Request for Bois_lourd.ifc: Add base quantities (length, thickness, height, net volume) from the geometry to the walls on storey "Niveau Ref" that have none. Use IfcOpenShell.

First a look at what the model holds.

```python
import ifcopenshell
import ifcopenshell.util.element
import ifcopenshell.util.unit

model = ifcopenshell.open("Bois_lourd.ifc")
print(model.schema)
for unit_type in ("LENGTHUNIT", "AREAUNIT", "VOLUMEUNIT"):
    print(unit_type, ifcopenshell.util.unit.calculate_unit_scale(model, unit_type))
storey = next(s for s in model.by_type("IfcBuildingStorey") if s.Name == "Niveau Ref")
walls = [e for e in ifcopenshell.util.element.get_decomposition(storey) if e.is_a("IfcWall")]
for e in sorted(walls, key=lambda e: e.id()):
    print(e.id(), e.is_a(), e.Name, list(ifcopenshell.util.element.get_psets(e, qtos_only=True)), sep=" | ")
```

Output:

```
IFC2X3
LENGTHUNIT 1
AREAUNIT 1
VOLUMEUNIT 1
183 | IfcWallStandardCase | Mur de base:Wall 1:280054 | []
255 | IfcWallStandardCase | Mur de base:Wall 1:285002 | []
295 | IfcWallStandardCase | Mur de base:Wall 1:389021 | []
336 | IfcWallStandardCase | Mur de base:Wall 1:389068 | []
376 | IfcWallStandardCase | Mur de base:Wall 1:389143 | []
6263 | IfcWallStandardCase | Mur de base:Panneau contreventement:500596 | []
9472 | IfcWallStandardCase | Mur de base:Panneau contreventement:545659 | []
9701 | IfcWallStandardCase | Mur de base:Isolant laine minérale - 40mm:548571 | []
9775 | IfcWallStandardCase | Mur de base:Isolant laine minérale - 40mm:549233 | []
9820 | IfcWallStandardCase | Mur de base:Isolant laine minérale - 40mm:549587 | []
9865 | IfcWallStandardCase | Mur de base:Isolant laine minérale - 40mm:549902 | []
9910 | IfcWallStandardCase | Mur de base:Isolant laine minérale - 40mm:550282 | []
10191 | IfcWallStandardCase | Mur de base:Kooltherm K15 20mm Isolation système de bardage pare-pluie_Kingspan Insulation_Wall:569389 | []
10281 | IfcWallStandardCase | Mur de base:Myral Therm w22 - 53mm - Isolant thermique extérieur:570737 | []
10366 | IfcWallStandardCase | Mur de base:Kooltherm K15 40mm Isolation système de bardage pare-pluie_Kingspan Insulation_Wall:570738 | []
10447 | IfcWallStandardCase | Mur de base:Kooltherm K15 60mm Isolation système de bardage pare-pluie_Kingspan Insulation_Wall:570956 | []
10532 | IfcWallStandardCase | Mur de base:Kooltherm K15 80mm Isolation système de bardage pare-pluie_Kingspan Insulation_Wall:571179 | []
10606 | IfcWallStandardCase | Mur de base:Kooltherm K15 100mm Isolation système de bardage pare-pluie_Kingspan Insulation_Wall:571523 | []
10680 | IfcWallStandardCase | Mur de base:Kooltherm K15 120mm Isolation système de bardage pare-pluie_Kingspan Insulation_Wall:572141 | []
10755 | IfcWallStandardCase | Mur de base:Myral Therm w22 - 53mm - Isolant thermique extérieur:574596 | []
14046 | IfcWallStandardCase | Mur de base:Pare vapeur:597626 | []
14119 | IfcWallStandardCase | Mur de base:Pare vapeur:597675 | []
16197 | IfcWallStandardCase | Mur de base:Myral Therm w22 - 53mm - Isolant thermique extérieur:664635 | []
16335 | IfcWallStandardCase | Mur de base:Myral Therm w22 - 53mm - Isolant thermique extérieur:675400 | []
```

```python
import ifcopenshell
import ifcopenshell.api.pset
import ifcopenshell.geom
import ifcopenshell.util.element
import ifcopenshell.util.shape
import ifcopenshell.util.unit

model = ifcopenshell.open("Bois_lourd.ifc")
unit_scale = ifcopenshell.util.unit.calculate_unit_scale(model)
volume_scale = ifcopenshell.util.unit.calculate_unit_scale(model, "VOLUMEUNIT")
settings = ifcopenshell.geom.settings()

storey = next(s for s in model.by_type("IfcBuildingStorey") if s.Name == "Niveau Ref")
walls = [e for e in ifcopenshell.util.element.get_decomposition(storey) if e.is_a("IfcWall")]

for e in sorted(walls, key=lambda e: e.id()):
    if ifcopenshell.util.element.get_psets(e, qtos_only=True, should_inherit=False):
        continue
    # Geometry comes back in metres, in the element's own axes.
    shape = ifcopenshell.geom.create_shape(settings, e)
    values = {
        "Length": ifcopenshell.util.shape.get_x(shape.geometry) / unit_scale,
        "Width": ifcopenshell.util.shape.get_y(shape.geometry) / unit_scale,
        "Height": ifcopenshell.util.shape.get_z(shape.geometry) / unit_scale,
        "NetVolume": ifcopenshell.util.shape.get_volume(shape.geometry) / volume_scale,
    }
    qto = ifcopenshell.api.pset.add_qto(model, product=e, name="BaseQuantities")
    ifcopenshell.api.pset.edit_qto(model, qto=qto, properties=values)
    print(e.id(), {k: round(v, 3) for k, v in values.items()})

model.write("Bois_lourd-out.ifc")
```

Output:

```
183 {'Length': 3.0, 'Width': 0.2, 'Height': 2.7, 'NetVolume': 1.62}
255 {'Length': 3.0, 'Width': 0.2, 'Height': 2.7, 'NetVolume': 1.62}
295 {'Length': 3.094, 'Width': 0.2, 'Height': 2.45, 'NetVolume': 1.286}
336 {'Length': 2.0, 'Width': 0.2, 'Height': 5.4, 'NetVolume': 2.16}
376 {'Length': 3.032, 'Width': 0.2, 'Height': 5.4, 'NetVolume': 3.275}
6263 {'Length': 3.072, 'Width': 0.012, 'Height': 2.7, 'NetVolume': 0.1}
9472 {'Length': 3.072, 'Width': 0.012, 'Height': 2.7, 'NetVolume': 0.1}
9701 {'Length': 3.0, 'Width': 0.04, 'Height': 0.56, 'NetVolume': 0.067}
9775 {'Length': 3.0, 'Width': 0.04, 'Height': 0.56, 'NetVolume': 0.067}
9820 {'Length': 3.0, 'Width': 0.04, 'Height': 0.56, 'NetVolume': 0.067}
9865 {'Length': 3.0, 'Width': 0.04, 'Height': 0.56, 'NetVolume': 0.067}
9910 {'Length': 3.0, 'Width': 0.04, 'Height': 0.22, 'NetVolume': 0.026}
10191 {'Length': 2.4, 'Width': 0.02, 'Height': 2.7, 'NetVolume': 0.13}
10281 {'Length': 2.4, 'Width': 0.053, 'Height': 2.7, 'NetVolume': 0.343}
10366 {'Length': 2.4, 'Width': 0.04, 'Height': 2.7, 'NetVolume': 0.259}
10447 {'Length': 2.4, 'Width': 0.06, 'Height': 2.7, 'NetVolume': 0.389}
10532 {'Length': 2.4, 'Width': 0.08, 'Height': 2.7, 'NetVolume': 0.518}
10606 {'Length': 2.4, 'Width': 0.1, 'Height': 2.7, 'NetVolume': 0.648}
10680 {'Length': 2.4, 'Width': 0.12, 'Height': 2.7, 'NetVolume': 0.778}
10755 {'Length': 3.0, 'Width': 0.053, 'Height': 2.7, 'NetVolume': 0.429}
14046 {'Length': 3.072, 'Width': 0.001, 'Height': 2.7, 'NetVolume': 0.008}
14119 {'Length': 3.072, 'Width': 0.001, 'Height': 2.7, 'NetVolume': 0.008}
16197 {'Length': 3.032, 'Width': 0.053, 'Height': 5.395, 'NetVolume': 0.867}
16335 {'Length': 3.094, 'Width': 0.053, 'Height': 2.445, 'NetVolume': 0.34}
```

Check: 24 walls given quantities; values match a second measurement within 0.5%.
